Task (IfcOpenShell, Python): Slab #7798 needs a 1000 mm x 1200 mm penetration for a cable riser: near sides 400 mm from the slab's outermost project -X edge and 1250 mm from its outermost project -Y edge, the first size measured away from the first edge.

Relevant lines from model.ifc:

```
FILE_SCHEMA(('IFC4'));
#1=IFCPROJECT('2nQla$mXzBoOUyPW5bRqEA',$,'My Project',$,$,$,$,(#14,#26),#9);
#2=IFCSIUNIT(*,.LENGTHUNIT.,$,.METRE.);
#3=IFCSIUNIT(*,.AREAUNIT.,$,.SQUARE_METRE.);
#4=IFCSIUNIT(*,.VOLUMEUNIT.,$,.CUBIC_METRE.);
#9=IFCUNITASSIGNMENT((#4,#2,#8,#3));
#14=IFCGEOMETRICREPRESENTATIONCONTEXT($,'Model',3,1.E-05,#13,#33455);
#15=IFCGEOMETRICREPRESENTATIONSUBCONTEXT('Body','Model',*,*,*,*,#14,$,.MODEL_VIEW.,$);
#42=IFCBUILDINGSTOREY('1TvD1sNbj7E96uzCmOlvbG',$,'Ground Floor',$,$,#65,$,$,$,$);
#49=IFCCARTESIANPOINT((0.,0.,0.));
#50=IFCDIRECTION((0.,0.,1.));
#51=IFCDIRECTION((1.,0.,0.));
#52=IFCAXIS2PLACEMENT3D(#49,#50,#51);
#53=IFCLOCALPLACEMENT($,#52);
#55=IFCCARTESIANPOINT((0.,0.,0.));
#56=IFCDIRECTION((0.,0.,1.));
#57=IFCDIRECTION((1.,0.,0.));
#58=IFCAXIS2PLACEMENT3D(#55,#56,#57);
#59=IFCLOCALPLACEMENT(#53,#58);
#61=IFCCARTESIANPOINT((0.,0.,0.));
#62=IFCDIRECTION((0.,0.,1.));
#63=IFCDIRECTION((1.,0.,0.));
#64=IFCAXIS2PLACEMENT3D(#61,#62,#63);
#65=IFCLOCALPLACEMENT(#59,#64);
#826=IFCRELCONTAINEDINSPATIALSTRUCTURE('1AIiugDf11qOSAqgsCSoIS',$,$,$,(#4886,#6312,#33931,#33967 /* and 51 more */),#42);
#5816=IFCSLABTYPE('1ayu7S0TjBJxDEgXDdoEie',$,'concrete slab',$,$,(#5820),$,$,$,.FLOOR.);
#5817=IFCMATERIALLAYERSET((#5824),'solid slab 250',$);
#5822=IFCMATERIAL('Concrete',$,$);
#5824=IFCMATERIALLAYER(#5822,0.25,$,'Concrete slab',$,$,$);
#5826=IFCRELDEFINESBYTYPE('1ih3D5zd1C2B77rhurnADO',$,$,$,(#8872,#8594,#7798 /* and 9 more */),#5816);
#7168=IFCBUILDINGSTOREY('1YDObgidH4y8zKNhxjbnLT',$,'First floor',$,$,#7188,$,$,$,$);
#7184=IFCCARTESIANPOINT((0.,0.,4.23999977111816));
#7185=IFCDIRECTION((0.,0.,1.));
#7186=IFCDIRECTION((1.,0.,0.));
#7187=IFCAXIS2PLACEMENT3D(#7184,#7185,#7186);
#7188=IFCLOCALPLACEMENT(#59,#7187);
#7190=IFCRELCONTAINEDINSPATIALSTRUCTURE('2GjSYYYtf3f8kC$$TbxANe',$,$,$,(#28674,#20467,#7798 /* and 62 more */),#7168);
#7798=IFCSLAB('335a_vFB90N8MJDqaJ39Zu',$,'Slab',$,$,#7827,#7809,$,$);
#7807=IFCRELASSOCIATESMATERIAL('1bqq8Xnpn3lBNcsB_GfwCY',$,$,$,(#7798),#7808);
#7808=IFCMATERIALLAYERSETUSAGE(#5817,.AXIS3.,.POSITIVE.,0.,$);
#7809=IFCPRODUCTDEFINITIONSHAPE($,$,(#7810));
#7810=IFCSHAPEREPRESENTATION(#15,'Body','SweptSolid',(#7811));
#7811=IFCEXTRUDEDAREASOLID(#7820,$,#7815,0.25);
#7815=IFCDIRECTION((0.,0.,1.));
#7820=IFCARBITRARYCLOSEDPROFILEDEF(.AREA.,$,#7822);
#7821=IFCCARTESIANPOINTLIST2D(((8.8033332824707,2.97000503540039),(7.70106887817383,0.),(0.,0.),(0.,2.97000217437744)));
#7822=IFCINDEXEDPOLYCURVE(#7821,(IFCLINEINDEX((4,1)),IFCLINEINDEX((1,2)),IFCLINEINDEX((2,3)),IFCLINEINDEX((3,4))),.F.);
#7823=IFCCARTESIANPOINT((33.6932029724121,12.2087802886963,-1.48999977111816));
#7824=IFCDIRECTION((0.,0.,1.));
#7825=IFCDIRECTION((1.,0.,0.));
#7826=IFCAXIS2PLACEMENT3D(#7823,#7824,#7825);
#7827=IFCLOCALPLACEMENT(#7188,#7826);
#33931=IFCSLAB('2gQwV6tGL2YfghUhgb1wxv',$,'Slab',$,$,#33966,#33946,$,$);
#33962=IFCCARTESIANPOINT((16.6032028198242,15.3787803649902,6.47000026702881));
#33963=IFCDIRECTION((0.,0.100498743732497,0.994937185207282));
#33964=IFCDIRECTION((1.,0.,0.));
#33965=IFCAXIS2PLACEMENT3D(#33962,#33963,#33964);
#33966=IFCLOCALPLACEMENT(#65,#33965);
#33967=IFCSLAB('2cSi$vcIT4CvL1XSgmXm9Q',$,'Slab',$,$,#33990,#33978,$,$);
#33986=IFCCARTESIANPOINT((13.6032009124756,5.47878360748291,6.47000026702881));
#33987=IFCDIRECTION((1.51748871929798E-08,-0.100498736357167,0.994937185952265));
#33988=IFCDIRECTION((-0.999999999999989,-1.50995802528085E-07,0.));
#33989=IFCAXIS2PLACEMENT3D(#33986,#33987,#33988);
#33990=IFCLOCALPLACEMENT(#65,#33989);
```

```python
import numpy as np
import ifcopenshell
import ifcopenshell.api.feature
import ifcopenshell.api.geometry
import ifcopenshell.api.root
import ifcopenshell.geom
import ifcopenshell.util.placement
import ifcopenshell.util.representation
import ifcopenshell.util.shape
import ifcopenshell.util.unit

model = ifcopenshell.open("model.ifc")
unit_scale = ifcopenshell.util.unit.calculate_unit_scale(model)
settings = ifcopenshell.geom.settings()


def volume(element):
    """Net volume in cubic metres, openings subtracted."""
    shape = ifcopenshell.geom.create_shape(settings, element)
    return ifcopenshell.util.shape.get_volume(shape.geometry)


slab = model.by_guid("335a_vFB90N8MJDqaJ39Zu")
before = volume(slab)

# Extent in the slab's own axes, in metres. The edges named are its -X and -Y sides.
slab_shape = ifcopenshell.geom.create_shape(settings, slab)
vertices = ifcopenshell.util.shape.get_vertices(slab_shape.geometry)
x_min, y_min, bottom = vertices.min(axis=0)
top = vertices[:, 2].max()

opening = ifcopenshell.api.root.create_entity(model, ifc_class="IfcOpeningElement", name="Cable riser opening", predefined_type="OPENING")
context = ifcopenshell.util.representation.get_context(model, "Model", "Body", "MODEL_VIEW")
width, depth = 1, 1.2
outline = [(0.0, 0.0), (width, 0.0), (width, depth), (0.0, depth), (0.0, 0.0)]
# Overshoot both faces by 50 mm so the cut is clean.
shape = ifcopenshell.api.geometry.add_slab_representation(
    model, context=context, depth=top - bottom + 0.1, polyline=outline
)
ifcopenshell.api.geometry.assign_representation(model, product=opening, representation=shape)

matrix = ifcopenshell.util.placement.get_local_placement(slab.ObjectPlacement)
matrix[:, 3] = matrix @ np.append(np.array([x_min + 0.4, y_min + 1.25, bottom - 0.05]) / unit_scale, 1.0)
ifcopenshell.api.geometry.edit_object_placement(model, product=opening, matrix=matrix, is_si=False)
ifcopenshell.api.feature.add_feature(model, feature=opening, element=slab)

after = volume(slab)

print(f"slab volume {before:.3f} -> {after:.3f} m3")

model.write("model_edited.ifc")
```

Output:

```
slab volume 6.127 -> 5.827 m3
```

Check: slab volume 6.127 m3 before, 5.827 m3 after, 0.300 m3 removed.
